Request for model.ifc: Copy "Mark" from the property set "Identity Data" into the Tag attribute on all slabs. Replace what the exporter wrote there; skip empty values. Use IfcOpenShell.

First a look at what the model holds.

```python
import ifcopenshell
import ifcopenshell.util.element

model = ifcopenshell.open("model.ifc")
print(model.schema)
slabs = model.by_type("IfcSlab")
print(len(slabs), "slabs")
for e in slabs[:8]:
    source = ifcopenshell.util.element.get_pset(e, "Identity Data", "Mark")
    target = e.Tag
    print(e.id(), repr(source), repr(target), sep=" | ")
```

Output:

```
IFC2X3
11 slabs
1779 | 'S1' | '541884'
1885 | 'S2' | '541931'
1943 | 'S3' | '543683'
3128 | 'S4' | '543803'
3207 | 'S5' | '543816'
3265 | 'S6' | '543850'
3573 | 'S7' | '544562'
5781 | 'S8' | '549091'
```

```python
import ifcopenshell
import ifcopenshell.util.element

model = ifcopenshell.open("model.ifc")

count = 0
for e in model.by_type("IfcSlab"):
    value = ifcopenshell.util.element.get_pset(e, "Identity Data", "Mark")
    current = e.Tag
    if not value or not value.strip() or current == value:
        continue
    e.Tag = value
    count += 1

print(count, "slabs updated")

model.write("model-out.ifc")
```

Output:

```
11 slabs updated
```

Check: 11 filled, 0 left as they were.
